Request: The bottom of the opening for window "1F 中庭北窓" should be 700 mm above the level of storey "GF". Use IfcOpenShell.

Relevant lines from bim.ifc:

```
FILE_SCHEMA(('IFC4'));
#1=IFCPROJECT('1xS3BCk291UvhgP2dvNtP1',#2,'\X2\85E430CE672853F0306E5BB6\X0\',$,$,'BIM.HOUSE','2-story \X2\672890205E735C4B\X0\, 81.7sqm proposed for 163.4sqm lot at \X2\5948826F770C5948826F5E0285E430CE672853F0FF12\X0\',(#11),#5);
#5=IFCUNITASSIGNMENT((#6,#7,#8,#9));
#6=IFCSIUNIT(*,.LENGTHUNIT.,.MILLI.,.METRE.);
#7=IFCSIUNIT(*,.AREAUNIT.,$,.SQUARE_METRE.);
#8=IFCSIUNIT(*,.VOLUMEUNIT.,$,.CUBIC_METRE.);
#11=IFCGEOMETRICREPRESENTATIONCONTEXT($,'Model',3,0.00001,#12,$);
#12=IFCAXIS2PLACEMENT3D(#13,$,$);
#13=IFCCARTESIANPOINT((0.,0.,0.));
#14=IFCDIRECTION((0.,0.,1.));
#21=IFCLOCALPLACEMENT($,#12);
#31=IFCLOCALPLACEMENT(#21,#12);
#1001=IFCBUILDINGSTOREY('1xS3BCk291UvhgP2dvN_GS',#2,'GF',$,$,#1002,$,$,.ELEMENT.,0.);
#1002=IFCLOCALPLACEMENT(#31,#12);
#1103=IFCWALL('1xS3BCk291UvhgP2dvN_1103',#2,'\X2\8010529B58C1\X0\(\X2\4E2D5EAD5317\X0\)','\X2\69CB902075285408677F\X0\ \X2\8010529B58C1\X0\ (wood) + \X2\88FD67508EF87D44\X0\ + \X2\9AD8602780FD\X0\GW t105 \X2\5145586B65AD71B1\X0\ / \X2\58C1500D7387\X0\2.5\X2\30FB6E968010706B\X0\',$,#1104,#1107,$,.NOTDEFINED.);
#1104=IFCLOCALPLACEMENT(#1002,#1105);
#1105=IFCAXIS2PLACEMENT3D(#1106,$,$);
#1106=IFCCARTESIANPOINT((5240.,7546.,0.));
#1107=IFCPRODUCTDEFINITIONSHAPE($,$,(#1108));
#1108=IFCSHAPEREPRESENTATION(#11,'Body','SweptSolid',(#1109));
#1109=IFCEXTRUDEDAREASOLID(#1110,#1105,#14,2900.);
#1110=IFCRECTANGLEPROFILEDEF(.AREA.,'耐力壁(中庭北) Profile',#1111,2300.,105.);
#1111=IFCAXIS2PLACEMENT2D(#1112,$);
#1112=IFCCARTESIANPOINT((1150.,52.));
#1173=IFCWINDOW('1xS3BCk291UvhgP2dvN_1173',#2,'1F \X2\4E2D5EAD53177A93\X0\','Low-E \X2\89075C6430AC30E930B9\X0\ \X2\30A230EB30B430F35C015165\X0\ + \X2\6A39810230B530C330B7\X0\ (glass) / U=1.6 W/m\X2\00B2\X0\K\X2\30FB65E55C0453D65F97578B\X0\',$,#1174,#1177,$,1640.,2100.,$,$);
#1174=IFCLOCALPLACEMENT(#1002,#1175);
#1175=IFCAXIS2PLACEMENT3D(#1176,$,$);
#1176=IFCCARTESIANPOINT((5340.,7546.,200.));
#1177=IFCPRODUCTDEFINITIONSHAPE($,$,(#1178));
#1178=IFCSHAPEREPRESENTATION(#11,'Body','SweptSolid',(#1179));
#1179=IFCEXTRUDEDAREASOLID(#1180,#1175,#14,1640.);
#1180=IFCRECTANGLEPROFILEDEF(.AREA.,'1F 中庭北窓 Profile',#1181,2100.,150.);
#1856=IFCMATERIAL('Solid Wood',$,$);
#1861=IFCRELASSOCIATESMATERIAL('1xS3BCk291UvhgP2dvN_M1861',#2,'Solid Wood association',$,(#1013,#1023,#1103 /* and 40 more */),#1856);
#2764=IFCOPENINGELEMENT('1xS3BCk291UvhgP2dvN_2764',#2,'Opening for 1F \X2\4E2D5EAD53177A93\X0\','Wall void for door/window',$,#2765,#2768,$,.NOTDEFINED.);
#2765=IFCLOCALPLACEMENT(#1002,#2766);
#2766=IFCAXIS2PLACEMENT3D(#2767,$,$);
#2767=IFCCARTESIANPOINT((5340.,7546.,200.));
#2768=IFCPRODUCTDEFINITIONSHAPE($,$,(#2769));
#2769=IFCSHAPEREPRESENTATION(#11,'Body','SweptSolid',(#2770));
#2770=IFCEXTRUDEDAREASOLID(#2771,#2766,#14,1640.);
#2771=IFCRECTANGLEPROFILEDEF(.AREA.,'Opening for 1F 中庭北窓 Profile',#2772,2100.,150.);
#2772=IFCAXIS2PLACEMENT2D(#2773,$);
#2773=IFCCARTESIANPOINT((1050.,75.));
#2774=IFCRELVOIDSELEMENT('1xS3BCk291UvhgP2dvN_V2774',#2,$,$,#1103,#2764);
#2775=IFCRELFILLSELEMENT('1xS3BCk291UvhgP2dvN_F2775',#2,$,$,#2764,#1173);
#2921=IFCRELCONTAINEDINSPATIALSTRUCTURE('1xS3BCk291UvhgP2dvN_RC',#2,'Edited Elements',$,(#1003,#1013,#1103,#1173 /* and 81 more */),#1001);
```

```python
import numpy as np
import ifcopenshell
import ifcopenshell.api.geometry
import ifcopenshell.geom
import ifcopenshell.util.element
import ifcopenshell.util.placement
import ifcopenshell.util.shape
import ifcopenshell.util.unit

model = ifcopenshell.open("bim.ifc")
unit_scale = ifcopenshell.util.unit.calculate_unit_scale(model)

window = model.by_guid("1xS3BCk291UvhgP2dvN_1173")
opening = window.FillsVoids[0].RelatingOpeningElement
storey = ifcopenshell.util.element.get_container(window, ifc_class="IfcBuildingStorey")
level = ifcopenshell.util.placement.get_local_placement(storey.ObjectPlacement)[2, 3]

# The opening's origin need not be at the sill, so measure its lowest point.
shape = ifcopenshell.geom.create_shape(ifcopenshell.geom.settings(), opening)
bottom = ifcopenshell.util.shape.get_shape_bottom_elevation(shape, shape.geometry) / unit_scale
dz = level + 0.7 / unit_scale - bottom

shift = np.array([0.0, 0.0, dz])
# The window is not placed relative to its opening, so move both.
for product in (opening, window):
    matrix = ifcopenshell.util.placement.get_local_placement(product.ObjectPlacement)
    matrix[:3, 3] += shift
    ifcopenshell.api.geometry.edit_object_placement(model, product=product, matrix=matrix, is_si=False)

print(f"moved by {dz * unit_scale:+.3f} m")

model.write("bim_v2.ifc")
```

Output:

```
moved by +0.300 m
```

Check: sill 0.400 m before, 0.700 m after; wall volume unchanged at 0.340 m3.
